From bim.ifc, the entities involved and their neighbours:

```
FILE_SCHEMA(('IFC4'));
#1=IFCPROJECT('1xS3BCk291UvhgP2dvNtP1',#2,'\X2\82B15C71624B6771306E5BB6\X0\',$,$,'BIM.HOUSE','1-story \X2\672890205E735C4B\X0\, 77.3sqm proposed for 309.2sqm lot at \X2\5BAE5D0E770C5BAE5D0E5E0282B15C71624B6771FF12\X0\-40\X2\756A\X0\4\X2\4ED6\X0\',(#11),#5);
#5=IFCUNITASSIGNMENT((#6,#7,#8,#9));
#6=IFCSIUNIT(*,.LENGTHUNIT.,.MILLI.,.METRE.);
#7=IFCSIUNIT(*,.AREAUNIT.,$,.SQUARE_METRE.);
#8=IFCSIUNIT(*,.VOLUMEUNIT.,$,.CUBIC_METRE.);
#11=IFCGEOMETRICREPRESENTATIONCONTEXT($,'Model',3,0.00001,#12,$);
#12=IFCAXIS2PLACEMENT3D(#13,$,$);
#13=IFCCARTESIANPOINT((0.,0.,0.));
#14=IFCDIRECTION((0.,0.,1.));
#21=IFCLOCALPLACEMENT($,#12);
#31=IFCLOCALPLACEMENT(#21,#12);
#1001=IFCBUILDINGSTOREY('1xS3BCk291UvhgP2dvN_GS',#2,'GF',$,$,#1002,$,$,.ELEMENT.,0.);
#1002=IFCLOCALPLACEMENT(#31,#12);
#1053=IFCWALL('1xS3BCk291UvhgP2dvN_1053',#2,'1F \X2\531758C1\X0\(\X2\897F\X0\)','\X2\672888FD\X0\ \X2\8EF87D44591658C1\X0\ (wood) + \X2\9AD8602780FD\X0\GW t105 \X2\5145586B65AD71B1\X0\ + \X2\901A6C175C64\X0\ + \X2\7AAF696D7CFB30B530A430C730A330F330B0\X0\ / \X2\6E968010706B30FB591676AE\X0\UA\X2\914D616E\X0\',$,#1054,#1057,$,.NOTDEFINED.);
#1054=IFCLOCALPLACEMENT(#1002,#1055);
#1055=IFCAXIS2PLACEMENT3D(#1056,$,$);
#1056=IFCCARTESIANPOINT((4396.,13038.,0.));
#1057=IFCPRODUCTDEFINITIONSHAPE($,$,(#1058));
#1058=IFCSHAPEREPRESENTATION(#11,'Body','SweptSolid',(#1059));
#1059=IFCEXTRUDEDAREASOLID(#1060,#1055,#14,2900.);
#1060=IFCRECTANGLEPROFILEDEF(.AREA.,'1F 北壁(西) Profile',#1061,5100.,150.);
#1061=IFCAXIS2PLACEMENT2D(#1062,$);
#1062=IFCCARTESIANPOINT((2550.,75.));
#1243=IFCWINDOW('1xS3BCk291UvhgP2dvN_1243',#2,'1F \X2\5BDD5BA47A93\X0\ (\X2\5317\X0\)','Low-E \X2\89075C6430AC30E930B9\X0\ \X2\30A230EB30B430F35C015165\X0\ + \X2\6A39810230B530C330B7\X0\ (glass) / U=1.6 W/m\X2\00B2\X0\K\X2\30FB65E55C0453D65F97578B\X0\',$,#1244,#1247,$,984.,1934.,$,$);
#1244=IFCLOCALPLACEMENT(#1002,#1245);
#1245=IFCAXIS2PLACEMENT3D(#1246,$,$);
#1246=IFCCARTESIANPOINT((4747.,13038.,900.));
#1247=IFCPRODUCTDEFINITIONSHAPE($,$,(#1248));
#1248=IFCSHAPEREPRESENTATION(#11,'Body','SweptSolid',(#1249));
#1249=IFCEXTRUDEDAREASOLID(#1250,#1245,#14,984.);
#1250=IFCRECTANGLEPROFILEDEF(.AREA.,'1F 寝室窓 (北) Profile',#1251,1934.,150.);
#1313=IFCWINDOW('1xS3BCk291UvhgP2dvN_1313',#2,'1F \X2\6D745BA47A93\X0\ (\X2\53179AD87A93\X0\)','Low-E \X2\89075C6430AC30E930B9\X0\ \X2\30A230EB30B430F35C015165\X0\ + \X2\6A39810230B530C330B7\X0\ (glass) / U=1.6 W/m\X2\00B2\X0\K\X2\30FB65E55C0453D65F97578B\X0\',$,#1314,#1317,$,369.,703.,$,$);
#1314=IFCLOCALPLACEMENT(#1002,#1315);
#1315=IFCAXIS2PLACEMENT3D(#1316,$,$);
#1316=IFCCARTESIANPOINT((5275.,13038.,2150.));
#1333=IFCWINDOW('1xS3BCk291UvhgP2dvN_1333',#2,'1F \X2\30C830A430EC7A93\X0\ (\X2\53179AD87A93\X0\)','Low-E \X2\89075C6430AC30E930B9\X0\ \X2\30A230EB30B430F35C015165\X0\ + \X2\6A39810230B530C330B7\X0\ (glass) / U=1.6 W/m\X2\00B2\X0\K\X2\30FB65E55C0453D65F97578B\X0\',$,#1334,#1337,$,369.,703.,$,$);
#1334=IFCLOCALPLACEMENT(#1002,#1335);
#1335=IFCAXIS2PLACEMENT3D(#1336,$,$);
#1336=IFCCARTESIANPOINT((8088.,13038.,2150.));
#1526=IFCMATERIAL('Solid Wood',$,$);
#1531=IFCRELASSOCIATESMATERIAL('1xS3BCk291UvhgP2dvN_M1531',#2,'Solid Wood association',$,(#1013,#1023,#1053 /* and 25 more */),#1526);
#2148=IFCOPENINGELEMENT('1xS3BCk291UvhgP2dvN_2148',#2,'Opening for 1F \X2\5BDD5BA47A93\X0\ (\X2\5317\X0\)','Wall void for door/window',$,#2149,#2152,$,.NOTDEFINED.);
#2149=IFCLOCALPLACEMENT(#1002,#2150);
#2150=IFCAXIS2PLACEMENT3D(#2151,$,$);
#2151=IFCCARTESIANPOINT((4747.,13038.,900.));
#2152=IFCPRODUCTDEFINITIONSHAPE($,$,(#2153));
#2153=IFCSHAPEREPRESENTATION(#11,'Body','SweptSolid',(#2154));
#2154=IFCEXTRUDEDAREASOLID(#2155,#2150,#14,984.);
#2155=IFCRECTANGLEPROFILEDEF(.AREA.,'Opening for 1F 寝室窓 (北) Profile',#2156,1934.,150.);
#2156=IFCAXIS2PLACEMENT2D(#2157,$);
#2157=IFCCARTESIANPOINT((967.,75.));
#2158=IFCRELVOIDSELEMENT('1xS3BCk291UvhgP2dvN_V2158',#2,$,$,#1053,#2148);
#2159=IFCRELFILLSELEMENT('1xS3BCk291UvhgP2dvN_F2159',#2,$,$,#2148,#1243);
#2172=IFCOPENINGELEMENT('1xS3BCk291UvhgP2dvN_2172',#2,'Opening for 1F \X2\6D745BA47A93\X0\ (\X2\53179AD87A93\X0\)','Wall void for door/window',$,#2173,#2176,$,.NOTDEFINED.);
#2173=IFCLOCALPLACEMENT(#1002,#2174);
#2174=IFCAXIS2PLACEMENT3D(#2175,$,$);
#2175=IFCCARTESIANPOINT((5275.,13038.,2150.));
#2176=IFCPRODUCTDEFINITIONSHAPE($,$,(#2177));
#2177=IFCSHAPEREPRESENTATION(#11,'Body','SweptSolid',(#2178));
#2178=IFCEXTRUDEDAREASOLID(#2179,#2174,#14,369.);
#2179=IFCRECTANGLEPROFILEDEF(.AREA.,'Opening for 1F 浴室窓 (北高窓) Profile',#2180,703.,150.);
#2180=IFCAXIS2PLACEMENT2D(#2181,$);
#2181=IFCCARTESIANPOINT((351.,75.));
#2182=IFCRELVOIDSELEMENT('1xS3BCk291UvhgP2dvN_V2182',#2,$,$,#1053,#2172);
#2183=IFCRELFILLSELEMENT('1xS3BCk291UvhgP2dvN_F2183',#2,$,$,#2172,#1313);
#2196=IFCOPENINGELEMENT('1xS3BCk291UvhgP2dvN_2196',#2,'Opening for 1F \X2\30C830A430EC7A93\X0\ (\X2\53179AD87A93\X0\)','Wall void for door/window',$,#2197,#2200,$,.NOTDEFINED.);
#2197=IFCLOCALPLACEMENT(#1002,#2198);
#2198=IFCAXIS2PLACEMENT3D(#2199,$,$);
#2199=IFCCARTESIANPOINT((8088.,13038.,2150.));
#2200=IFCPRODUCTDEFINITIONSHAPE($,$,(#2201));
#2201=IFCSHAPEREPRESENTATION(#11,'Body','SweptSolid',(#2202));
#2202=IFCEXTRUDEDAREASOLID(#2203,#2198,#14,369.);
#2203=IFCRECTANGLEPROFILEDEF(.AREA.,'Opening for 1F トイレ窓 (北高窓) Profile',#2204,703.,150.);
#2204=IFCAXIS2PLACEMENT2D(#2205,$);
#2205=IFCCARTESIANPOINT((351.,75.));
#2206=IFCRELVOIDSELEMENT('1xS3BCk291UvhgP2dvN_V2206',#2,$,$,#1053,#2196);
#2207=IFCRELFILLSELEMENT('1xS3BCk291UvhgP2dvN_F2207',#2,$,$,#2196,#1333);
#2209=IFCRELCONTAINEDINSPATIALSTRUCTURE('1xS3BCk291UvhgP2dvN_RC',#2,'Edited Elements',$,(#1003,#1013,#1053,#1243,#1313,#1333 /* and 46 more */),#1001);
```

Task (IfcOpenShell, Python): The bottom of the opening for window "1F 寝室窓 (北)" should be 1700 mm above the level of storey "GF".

```python
import numpy as np
import ifcopenshell
import ifcopenshell.api.geometry
import ifcopenshell.geom
import ifcopenshell.util.element
import ifcopenshell.util.placement
import ifcopenshell.util.shape
import ifcopenshell.util.unit

model = ifcopenshell.open("bim.ifc")
unit_scale = ifcopenshell.util.unit.calculate_unit_scale(model)

window = model.by_guid("1xS3BCk291UvhgP2dvN_1243")
opening = window.FillsVoids[0].RelatingOpeningElement
storey = ifcopenshell.util.element.get_container(window, ifc_class="IfcBuildingStorey")
level = ifcopenshell.util.placement.get_local_placement(storey.ObjectPlacement)[2, 3]

# The opening's origin need not be at the sill, so measure its lowest point.
shape = ifcopenshell.geom.create_shape(ifcopenshell.geom.settings(), opening)
bottom = ifcopenshell.util.shape.get_shape_bottom_elevation(shape, shape.geometry) / unit_scale
dz = level + 1700.0 - bottom

shift = np.array([0.0, 0.0, dz])
# The window is not placed relative to its opening, so move both.
for product in (opening, window):
    matrix = ifcopenshell.util.placement.get_local_placement(product.ObjectPlacement)
    matrix[:3, 3] += shift
    ifcopenshell.api.geometry.edit_object_placement(model, product=product, matrix=matrix, is_si=False)

print(f"moved by {dz * unit_scale:+.3f} m")

model.write("bim_updated.ifc")
```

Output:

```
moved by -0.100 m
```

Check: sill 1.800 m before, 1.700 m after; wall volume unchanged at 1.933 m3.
